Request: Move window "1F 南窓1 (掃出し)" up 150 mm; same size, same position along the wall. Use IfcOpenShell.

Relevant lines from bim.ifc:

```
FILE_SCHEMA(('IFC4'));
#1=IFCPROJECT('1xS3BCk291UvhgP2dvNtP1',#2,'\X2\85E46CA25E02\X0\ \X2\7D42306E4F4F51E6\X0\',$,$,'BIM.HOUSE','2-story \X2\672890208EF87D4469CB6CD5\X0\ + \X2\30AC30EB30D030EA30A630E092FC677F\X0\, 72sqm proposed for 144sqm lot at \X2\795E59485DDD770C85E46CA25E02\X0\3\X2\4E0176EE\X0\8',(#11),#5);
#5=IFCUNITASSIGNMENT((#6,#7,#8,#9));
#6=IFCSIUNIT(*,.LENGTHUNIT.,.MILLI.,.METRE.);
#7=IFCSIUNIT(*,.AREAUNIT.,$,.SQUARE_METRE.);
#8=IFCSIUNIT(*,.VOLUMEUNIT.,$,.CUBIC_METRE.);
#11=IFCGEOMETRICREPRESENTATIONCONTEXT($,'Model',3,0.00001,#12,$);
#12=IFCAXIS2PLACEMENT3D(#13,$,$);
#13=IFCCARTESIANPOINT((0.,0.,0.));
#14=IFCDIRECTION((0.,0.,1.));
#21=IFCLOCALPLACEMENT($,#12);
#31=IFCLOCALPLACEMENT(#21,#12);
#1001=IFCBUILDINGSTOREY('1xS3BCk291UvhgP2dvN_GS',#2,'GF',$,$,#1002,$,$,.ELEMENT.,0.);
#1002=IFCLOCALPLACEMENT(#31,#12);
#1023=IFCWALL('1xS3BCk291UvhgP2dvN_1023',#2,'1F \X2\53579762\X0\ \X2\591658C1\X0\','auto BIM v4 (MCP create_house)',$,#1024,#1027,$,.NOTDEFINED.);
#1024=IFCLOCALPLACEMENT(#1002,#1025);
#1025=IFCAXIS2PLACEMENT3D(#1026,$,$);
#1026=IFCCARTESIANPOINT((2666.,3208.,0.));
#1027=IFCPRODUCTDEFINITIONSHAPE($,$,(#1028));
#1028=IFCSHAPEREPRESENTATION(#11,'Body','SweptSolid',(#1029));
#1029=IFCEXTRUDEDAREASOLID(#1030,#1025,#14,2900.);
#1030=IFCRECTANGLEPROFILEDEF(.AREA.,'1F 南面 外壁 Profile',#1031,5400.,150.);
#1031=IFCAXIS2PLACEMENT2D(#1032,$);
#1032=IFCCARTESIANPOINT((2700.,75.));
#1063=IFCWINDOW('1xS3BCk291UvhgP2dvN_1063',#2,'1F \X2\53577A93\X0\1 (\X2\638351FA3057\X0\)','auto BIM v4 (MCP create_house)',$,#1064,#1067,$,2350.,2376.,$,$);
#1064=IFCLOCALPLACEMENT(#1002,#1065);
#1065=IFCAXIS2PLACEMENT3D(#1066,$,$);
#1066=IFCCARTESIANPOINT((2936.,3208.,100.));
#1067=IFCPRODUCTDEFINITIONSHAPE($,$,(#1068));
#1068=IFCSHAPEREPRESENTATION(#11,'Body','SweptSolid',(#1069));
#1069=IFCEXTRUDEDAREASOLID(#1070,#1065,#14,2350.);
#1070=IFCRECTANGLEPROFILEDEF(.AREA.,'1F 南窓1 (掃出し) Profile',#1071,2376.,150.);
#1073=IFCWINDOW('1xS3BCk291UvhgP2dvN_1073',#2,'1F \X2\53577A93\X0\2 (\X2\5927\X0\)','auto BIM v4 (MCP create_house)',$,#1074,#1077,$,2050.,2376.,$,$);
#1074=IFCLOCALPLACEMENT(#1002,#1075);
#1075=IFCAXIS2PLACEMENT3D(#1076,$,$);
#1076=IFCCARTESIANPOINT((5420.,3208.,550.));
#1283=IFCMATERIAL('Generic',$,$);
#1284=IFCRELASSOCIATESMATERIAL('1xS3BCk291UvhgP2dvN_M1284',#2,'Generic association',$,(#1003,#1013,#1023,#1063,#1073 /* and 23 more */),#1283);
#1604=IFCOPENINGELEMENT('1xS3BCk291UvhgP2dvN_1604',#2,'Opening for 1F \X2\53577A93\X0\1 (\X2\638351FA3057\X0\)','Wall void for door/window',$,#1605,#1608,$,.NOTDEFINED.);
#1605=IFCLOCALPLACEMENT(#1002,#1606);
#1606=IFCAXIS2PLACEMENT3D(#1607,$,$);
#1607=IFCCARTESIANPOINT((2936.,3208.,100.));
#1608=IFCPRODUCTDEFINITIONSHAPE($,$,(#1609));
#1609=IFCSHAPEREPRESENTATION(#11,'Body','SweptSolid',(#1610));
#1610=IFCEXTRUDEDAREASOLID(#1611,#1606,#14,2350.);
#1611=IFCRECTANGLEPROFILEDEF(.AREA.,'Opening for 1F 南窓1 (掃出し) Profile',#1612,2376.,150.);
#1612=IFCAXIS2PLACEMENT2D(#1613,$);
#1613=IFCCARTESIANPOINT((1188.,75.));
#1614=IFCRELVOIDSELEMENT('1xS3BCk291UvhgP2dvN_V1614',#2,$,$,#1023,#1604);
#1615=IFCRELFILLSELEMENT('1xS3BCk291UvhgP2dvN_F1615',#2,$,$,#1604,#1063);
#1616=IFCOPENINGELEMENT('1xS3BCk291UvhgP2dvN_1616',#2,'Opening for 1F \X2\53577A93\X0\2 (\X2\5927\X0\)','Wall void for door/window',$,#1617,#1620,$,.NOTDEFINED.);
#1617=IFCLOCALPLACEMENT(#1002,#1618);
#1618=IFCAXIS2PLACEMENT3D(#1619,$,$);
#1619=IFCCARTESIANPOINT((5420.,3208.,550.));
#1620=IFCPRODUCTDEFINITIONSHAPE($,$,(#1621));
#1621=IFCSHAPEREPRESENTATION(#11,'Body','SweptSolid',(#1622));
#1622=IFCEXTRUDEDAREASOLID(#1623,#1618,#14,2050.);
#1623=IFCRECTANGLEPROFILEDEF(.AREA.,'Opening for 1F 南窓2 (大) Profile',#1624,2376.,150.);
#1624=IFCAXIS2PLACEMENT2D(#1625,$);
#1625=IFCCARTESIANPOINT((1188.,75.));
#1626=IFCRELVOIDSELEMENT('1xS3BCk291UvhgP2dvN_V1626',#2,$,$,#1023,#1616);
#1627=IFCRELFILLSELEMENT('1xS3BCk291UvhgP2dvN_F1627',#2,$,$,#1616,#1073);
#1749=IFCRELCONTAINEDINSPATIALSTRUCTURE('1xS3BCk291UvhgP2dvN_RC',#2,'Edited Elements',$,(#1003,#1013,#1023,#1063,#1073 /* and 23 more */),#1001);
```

```python
import numpy as np
import ifcopenshell
import ifcopenshell.api.geometry
import ifcopenshell.util.placement
import ifcopenshell.util.unit

model = ifcopenshell.open("bim.ifc")
unit_scale = ifcopenshell.util.unit.calculate_unit_scale(model)

window = model.by_guid("1xS3BCk291UvhgP2dvN_1063")
opening = window.FillsVoids[0].RelatingOpeningElement
dz = 0.15 / unit_scale

shift = np.array([0.0, 0.0, dz])
# The window is not placed relative to its opening, so move both.
for product in (opening, window):
    matrix = ifcopenshell.util.placement.get_local_placement(product.ObjectPlacement)
    matrix[:3, 3] += shift
    ifcopenshell.api.geometry.edit_object_placement(model, product=product, matrix=matrix, is_si=False)

print(f"moved by {dz * unit_scale:+.3f} m")

model.write("bim_rev.ifc")
```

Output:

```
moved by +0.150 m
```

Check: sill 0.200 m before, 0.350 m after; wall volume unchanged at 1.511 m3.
